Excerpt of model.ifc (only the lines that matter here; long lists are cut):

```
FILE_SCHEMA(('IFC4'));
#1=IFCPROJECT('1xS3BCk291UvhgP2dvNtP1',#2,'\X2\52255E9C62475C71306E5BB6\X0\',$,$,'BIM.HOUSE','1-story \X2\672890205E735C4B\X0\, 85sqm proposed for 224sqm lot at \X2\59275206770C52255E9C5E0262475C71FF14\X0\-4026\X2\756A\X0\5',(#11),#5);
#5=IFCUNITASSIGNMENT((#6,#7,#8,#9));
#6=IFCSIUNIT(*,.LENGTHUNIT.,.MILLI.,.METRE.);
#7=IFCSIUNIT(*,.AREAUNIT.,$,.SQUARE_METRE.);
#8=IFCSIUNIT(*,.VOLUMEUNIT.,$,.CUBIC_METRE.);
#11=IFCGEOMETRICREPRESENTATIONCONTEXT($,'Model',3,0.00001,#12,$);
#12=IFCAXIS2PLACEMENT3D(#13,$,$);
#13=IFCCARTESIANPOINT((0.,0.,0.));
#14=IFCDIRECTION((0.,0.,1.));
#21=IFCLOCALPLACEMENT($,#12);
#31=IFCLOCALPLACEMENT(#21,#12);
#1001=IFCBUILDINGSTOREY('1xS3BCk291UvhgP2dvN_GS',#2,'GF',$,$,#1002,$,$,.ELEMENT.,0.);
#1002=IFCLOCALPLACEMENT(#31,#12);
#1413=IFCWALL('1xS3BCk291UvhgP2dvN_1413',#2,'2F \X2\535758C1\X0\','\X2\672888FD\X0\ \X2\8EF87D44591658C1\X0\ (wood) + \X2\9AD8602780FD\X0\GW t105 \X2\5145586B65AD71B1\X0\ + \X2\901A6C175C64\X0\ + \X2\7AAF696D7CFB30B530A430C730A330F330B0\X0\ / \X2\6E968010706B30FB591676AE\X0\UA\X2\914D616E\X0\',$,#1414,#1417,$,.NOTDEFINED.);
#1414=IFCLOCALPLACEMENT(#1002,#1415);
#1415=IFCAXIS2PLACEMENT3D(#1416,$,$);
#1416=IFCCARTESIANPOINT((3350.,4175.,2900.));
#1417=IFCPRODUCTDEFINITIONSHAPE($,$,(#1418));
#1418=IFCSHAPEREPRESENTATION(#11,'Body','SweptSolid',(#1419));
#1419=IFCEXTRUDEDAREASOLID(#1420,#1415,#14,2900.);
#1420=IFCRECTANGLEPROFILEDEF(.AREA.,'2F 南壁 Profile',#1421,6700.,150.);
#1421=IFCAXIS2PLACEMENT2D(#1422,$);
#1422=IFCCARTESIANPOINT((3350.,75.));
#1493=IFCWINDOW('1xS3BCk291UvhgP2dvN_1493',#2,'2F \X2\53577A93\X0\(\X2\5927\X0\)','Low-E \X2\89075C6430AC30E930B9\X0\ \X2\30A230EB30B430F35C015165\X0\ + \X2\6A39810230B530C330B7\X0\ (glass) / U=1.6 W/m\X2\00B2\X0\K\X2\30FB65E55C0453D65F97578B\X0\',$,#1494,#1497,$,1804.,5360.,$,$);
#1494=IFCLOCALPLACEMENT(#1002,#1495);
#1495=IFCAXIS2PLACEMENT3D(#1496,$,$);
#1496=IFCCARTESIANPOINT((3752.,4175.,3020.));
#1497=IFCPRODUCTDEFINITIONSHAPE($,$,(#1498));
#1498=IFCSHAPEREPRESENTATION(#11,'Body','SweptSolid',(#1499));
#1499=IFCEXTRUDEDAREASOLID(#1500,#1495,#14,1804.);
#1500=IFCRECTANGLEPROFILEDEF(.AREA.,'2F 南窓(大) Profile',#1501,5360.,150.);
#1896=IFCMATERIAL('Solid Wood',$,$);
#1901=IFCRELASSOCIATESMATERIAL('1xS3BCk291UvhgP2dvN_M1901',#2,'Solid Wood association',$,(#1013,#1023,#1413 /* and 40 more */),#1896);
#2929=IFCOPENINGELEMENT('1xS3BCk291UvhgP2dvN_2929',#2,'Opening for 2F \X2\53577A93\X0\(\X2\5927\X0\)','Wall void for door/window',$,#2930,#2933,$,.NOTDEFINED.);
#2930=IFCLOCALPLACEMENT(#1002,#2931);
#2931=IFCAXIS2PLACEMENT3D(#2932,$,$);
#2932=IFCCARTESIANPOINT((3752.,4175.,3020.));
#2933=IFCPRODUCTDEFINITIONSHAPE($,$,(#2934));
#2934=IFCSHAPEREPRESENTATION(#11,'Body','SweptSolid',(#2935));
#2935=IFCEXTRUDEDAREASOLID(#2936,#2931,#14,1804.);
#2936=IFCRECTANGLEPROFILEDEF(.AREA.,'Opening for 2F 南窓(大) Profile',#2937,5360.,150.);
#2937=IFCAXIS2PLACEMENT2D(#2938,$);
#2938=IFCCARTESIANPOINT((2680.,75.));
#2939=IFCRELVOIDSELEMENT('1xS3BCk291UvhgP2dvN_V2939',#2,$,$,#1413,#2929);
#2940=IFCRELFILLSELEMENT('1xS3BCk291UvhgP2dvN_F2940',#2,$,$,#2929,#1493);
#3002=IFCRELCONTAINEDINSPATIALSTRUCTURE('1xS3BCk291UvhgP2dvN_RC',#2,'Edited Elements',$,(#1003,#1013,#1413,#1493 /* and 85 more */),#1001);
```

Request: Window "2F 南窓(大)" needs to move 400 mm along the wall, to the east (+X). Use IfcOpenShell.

```python
import ifcopenshell
import ifcopenshell.api.geometry
import ifcopenshell.util.placement
import ifcopenshell.util.unit

model = ifcopenshell.open("model.ifc")
unit_scale = ifcopenshell.util.unit.calculate_unit_scale(model)

window = model.by_guid("1xS3BCk291UvhgP2dvN_1493")
opening = window.FillsVoids[0].RelatingOpeningElement
wall = opening.VoidsElements[0].RelatingBuildingElement

wall_matrix = ifcopenshell.util.placement.get_local_placement(wall.ObjectPlacement)
shift = wall_matrix[:3, 0] * 0.4 / unit_scale
before = ifcopenshell.util.placement.get_local_placement(window.ObjectPlacement)[:3, 3].copy()

# The window is not placed relative to its opening, so move both.
for product in (opening, window):
    matrix = ifcopenshell.util.placement.get_local_placement(product.ObjectPlacement)
    matrix[:3, 3] += shift
    ifcopenshell.api.geometry.edit_object_placement(model, product=product, matrix=matrix, is_si=False)

after = ifcopenshell.util.placement.get_local_placement(window.ObjectPlacement)[:3, 3]
print("window moved by", (after - before).round(3) + 0.0)

model.write("model-out.ifc")
```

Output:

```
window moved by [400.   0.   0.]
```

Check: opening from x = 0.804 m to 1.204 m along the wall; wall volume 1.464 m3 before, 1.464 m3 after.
